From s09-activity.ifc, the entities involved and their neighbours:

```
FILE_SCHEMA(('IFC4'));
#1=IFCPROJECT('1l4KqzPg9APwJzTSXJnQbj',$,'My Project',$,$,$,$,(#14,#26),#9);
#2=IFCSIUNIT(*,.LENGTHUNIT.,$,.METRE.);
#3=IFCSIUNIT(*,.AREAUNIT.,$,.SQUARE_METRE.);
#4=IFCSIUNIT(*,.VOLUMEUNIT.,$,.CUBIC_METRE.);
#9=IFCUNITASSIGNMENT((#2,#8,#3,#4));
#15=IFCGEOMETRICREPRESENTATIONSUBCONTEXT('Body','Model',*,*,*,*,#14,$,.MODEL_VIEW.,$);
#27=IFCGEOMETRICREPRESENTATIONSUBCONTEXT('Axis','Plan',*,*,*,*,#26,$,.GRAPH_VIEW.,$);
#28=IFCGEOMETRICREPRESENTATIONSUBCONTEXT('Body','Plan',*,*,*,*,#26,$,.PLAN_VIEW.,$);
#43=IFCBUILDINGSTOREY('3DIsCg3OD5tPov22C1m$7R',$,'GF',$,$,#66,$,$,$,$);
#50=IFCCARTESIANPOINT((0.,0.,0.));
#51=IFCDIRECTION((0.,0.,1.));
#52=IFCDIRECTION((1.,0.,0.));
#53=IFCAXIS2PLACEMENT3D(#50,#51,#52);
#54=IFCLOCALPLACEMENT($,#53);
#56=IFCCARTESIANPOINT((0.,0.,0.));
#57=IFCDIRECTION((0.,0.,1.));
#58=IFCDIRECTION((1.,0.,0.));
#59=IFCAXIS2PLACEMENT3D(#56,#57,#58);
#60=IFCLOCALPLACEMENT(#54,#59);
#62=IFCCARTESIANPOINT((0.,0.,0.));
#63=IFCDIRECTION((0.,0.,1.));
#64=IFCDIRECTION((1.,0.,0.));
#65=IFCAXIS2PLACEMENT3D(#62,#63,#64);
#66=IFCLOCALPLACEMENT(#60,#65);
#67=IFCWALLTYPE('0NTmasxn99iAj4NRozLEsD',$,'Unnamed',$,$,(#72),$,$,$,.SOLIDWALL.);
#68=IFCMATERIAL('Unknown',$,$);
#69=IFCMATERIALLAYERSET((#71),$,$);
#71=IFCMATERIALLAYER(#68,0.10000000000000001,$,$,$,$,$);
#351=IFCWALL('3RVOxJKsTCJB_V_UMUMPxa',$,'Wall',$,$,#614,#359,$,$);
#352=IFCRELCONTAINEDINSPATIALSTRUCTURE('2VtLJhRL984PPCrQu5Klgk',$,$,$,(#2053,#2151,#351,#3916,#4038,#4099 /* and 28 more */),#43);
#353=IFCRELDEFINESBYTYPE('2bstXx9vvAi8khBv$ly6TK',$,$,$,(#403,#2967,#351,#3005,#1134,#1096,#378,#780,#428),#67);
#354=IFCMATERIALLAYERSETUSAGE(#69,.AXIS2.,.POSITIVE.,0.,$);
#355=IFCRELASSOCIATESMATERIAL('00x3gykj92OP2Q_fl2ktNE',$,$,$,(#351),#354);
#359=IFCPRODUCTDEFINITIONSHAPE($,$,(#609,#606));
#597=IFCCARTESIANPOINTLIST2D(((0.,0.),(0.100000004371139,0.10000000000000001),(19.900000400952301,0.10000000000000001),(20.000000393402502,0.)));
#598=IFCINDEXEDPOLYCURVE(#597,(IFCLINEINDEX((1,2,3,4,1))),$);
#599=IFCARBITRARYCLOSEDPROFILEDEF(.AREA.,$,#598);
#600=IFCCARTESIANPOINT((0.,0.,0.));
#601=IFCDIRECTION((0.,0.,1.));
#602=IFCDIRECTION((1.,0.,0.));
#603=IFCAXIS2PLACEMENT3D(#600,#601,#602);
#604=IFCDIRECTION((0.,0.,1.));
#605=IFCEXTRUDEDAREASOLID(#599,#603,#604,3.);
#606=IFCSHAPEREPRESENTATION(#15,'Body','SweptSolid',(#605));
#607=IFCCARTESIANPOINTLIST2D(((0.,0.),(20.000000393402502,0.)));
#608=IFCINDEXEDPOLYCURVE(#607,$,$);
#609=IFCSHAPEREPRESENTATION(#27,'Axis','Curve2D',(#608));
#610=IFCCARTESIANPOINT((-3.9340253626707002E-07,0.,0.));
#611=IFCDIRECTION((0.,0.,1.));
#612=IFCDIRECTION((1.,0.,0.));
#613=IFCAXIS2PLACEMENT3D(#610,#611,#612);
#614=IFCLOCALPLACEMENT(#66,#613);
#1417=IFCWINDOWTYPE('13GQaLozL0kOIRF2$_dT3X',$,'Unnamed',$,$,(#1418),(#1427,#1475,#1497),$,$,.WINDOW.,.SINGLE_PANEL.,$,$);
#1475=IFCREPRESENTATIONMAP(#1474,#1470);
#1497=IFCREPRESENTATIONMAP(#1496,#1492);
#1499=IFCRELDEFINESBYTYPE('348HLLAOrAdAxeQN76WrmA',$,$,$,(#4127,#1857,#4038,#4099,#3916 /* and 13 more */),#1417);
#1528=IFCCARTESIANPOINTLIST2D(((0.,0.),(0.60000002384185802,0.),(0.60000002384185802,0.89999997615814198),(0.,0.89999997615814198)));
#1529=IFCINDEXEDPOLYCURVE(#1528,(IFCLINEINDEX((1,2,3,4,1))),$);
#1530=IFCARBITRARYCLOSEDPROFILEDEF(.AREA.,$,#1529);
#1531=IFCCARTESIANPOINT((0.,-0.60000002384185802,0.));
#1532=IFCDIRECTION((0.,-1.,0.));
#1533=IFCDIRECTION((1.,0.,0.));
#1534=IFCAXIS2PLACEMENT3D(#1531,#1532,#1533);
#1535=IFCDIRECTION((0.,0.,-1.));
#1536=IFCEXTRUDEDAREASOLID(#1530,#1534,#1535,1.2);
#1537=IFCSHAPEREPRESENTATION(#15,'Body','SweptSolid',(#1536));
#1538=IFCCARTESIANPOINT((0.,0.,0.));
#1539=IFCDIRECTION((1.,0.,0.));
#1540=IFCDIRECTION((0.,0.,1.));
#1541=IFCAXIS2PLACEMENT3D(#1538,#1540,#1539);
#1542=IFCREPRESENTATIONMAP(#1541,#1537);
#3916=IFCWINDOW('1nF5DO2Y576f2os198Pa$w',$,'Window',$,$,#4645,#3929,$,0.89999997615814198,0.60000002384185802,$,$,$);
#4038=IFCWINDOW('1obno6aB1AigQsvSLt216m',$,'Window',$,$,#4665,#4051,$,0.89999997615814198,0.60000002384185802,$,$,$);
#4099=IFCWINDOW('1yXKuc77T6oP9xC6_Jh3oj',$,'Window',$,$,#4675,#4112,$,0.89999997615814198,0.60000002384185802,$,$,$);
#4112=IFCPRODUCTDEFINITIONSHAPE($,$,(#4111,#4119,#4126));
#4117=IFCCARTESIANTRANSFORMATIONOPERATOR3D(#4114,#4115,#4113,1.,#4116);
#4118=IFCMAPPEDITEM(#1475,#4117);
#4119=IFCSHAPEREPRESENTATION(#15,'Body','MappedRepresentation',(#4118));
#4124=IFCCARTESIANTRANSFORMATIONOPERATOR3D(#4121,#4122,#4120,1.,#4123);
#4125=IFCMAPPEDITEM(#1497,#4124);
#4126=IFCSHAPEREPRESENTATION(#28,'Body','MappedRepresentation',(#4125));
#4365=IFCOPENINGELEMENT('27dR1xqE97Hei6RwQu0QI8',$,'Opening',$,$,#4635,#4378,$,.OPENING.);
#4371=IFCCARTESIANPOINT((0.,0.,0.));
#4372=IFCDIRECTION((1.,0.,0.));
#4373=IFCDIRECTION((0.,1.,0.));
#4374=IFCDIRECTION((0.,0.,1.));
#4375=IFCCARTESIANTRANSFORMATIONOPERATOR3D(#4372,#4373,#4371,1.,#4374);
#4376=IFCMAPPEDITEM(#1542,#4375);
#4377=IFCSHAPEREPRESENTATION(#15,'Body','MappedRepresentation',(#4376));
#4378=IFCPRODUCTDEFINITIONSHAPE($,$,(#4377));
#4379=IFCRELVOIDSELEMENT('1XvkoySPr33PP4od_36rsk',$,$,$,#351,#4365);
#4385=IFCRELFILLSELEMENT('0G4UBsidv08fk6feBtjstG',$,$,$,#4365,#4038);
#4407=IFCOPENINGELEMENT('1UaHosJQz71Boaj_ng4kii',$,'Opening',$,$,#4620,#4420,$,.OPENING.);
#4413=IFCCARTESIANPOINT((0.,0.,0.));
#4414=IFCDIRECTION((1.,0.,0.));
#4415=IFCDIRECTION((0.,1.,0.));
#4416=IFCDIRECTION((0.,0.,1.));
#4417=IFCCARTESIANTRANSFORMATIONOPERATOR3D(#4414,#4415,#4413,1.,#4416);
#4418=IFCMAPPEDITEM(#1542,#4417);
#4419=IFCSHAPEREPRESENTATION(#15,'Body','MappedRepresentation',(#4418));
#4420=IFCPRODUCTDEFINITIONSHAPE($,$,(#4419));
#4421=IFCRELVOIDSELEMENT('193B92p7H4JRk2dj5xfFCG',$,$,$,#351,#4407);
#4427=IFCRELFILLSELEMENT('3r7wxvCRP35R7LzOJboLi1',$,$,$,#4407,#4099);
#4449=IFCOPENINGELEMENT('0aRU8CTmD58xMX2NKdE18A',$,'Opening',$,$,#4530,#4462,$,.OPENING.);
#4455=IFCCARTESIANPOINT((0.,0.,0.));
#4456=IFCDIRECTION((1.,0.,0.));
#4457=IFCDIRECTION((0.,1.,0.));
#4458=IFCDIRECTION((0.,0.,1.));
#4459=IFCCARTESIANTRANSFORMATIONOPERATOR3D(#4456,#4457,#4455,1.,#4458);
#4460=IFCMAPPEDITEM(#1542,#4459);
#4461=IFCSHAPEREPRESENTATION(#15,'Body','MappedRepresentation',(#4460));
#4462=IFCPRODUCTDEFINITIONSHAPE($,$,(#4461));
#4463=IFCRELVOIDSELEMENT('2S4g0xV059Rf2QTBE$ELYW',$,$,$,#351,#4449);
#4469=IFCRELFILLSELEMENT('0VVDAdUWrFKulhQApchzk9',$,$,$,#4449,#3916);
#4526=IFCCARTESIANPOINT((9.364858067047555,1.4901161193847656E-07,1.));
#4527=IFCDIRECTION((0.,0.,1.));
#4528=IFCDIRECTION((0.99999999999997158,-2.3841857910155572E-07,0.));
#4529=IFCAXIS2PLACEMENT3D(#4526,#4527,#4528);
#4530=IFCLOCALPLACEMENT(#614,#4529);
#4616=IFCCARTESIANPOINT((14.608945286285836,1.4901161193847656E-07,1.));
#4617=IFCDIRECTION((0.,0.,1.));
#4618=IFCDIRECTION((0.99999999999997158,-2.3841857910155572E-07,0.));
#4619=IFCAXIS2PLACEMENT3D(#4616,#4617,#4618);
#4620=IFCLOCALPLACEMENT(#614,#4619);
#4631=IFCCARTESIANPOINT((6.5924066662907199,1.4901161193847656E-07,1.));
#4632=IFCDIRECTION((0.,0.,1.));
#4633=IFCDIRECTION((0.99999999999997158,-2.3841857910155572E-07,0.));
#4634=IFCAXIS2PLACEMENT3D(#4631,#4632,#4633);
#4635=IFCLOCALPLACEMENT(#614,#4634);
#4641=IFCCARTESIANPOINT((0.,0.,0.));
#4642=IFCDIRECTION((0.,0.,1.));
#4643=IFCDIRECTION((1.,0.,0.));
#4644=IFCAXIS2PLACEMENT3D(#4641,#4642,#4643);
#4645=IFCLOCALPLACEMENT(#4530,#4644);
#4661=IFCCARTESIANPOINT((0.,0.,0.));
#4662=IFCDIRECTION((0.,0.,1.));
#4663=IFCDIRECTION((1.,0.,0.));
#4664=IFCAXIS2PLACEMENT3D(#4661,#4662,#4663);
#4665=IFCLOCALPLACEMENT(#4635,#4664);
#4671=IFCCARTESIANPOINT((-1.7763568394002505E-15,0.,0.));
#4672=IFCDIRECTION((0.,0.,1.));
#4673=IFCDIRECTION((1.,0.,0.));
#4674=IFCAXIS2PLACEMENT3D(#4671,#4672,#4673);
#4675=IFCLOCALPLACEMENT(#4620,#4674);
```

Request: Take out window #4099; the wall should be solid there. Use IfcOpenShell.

```python
import ifcopenshell
import ifcopenshell.api.feature
import ifcopenshell.api.root
import ifcopenshell.geom
import ifcopenshell.util.shape

model = ifcopenshell.open("s09-activity.ifc")
settings = ifcopenshell.geom.settings()


def volume(element):
    """Net volume in cubic metres, openings subtracted."""
    shape = ifcopenshell.geom.create_shape(settings, element)
    return ifcopenshell.util.shape.get_volume(shape.geometry)


window = model.by_guid("1yXKuc77T6oP9xC6_Jh3oj")
opening = window.FillsVoids[0].RelatingOpeningElement
wall = opening.VoidsElements[0].RelatingBuildingElement
before = volume(wall)

ifcopenshell.api.root.remove_product(model, product=window)
ifcopenshell.api.feature.remove_feature(model, feature=opening)

after = volume(wall)

print(f"wall volume {before:.3f} -> {after:.3f} m3")

model.write("s09-activity_v2.ifc")
```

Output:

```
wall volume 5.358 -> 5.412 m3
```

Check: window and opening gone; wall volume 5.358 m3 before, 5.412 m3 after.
